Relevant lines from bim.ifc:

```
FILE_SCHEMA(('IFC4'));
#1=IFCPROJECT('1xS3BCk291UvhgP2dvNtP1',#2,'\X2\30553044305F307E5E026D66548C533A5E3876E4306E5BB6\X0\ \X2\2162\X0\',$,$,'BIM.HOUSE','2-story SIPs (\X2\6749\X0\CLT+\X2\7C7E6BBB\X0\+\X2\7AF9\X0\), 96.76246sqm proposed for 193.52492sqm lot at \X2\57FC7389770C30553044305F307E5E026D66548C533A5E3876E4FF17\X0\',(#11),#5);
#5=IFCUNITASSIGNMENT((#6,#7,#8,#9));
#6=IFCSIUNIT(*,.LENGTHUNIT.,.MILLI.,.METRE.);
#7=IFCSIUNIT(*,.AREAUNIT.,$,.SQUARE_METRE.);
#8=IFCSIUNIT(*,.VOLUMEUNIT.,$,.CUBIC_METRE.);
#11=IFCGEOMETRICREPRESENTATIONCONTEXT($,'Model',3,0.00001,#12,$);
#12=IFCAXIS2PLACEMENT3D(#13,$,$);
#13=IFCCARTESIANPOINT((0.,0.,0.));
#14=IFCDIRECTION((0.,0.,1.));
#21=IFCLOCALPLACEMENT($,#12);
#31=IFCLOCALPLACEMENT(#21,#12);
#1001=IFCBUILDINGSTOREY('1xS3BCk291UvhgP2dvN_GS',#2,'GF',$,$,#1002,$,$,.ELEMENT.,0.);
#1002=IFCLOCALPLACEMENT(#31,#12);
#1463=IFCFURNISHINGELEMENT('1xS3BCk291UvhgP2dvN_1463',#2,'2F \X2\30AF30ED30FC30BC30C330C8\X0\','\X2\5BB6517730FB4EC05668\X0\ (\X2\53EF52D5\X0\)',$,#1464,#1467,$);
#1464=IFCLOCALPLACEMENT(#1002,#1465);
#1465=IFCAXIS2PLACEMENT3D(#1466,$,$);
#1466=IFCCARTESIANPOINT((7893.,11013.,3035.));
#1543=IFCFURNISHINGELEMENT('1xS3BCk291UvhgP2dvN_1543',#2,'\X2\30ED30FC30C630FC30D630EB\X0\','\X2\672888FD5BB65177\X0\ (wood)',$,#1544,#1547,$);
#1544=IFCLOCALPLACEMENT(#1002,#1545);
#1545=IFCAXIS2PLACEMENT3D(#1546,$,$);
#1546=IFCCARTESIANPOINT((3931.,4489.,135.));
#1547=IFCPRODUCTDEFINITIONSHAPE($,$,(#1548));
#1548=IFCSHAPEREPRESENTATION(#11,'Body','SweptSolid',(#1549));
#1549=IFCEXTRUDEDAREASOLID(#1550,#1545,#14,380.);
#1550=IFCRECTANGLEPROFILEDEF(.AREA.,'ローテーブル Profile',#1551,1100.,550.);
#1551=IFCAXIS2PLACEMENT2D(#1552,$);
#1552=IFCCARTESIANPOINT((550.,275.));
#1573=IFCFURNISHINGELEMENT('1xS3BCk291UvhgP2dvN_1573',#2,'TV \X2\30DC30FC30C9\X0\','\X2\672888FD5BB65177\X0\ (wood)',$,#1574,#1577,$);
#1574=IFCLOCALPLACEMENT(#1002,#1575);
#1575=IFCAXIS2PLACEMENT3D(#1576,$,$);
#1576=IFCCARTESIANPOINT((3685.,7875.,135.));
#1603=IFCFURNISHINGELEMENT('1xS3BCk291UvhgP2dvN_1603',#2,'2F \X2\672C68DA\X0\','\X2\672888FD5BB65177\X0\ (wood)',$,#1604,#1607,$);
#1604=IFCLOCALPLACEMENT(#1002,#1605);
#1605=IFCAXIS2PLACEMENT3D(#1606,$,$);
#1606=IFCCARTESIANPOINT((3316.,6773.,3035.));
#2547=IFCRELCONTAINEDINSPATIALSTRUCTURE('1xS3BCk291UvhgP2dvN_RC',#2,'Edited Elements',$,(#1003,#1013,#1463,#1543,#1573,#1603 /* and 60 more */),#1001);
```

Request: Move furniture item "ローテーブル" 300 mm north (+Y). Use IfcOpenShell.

```python
import ifcopenshell
import ifcopenshell.api.geometry
import ifcopenshell.util.placement
import ifcopenshell.util.unit

model = ifcopenshell.open("bim.ifc")
unit_scale = ifcopenshell.util.unit.calculate_unit_scale(model)

item = model.by_guid("1xS3BCk291UvhgP2dvN_1543")
matrix = ifcopenshell.util.placement.get_local_placement(item.ObjectPlacement)
matrix[1, 3] += 0.3 / unit_scale
ifcopenshell.api.geometry.edit_object_placement(model, product=item, matrix=matrix, is_si=False)

print(ifcopenshell.util.placement.get_local_placement(item.ObjectPlacement).round(3) + 0.0)

model.write("bim_edited.ifc")
```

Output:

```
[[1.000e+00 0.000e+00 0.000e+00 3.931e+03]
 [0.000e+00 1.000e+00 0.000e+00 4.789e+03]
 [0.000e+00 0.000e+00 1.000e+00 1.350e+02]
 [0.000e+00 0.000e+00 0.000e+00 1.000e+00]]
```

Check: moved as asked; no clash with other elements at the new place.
